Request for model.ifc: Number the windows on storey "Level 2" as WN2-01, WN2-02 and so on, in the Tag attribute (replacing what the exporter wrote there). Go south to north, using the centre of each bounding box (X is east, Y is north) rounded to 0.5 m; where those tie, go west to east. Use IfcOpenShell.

First a look at what the model holds.

```python
import ifcopenshell
import ifcopenshell.util.element
import ifcopenshell.util.placement

model = ifcopenshell.open("model.ifc")
print(model.schema)
storey = next(s for s in model.by_type("IfcBuildingStorey") if s.Name == "Level 2")
windows = [e for e in ifcopenshell.util.element.get_decomposition(storey) if e.is_a("IfcWindow")]
for e in sorted(windows, key=lambda e: e.id()):
    origin = ifcopenshell.util.placement.get_local_placement(e.ObjectPlacement)[:3, 3]
    print(e.id(), e.Tag, e.Name, origin.round(2) + 0.0, sep=" | ")
```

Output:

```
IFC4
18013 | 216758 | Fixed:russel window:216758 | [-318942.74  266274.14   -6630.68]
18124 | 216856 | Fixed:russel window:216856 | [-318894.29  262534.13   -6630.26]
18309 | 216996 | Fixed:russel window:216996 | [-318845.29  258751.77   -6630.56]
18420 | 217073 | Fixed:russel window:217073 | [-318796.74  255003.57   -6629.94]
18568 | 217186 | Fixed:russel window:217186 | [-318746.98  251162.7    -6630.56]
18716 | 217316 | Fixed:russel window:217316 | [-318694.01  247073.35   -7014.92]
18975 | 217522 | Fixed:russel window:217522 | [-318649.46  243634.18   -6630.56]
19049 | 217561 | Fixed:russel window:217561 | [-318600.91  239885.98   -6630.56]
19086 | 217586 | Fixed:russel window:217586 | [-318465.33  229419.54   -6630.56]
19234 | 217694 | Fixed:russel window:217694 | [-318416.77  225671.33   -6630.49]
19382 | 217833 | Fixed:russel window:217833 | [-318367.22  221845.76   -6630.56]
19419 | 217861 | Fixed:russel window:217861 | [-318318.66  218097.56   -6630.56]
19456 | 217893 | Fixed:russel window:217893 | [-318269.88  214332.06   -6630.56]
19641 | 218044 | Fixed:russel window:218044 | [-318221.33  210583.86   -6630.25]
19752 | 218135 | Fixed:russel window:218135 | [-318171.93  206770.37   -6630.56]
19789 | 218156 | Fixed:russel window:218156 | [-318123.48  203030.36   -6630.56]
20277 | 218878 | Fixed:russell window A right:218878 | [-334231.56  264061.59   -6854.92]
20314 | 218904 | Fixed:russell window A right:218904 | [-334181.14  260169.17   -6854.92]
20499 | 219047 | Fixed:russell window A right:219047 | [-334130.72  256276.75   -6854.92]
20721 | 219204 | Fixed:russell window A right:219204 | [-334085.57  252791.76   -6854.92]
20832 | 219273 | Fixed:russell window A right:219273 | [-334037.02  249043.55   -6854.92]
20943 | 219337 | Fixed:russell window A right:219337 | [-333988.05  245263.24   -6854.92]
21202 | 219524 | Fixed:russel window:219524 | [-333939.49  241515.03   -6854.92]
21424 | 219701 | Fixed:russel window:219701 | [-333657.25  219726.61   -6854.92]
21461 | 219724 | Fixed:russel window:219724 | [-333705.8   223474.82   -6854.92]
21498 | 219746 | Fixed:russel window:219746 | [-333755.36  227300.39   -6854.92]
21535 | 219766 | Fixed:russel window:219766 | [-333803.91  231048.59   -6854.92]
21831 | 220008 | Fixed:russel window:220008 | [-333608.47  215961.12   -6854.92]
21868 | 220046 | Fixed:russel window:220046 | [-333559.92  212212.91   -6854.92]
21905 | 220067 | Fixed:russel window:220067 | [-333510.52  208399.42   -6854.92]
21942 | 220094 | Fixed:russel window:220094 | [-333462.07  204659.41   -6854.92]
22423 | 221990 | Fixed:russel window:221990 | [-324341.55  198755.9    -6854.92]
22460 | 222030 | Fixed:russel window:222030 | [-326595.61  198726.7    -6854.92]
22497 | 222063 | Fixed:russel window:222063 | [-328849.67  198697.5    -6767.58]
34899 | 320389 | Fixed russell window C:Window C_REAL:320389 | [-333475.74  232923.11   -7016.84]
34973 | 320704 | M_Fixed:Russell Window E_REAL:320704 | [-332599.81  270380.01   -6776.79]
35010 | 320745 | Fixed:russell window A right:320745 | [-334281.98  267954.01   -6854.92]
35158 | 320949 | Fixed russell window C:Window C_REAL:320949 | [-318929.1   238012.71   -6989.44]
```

```python
import ifcopenshell
import ifcopenshell.geom
import ifcopenshell.util.element
import ifcopenshell.util.shape

model = ifcopenshell.open("model.ifc")
settings = ifcopenshell.geom.settings()
settings.set("use-world-coords", True)


def centre(element):
    shape = ifcopenshell.geom.create_shape(settings, element)
    return ifcopenshell.util.shape.get_bbox_centroid(shape.geometry)


storey = next(s for s in model.by_type("IfcBuildingStorey") if s.Name == "Level 2")
windows = [e for e in ifcopenshell.util.element.get_decomposition(storey) if e.is_a("IfcWindow")]

# Insertion points can sit at a corner or the storey origin, so sort by the geometry (in metres).
centres = {e: centre(e) for e in windows}
windows.sort(key=lambda e: (round(centres[e][1] / 0.5), centres[e][0]))

for i, e in enumerate(windows, start=1):
    number = f"WN2-{i:02d}"
    e.Tag = number
    print(e.id(), number)

model.write("model_updated.ifc")
```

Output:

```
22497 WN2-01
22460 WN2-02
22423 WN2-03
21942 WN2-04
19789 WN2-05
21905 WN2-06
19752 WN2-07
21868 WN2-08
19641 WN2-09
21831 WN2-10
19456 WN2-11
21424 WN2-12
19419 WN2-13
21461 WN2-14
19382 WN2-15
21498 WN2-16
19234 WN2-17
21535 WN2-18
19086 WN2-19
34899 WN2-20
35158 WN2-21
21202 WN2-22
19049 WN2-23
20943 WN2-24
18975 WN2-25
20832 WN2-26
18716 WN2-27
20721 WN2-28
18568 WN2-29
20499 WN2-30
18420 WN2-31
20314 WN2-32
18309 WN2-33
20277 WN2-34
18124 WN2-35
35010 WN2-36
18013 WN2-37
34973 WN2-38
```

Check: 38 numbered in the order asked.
